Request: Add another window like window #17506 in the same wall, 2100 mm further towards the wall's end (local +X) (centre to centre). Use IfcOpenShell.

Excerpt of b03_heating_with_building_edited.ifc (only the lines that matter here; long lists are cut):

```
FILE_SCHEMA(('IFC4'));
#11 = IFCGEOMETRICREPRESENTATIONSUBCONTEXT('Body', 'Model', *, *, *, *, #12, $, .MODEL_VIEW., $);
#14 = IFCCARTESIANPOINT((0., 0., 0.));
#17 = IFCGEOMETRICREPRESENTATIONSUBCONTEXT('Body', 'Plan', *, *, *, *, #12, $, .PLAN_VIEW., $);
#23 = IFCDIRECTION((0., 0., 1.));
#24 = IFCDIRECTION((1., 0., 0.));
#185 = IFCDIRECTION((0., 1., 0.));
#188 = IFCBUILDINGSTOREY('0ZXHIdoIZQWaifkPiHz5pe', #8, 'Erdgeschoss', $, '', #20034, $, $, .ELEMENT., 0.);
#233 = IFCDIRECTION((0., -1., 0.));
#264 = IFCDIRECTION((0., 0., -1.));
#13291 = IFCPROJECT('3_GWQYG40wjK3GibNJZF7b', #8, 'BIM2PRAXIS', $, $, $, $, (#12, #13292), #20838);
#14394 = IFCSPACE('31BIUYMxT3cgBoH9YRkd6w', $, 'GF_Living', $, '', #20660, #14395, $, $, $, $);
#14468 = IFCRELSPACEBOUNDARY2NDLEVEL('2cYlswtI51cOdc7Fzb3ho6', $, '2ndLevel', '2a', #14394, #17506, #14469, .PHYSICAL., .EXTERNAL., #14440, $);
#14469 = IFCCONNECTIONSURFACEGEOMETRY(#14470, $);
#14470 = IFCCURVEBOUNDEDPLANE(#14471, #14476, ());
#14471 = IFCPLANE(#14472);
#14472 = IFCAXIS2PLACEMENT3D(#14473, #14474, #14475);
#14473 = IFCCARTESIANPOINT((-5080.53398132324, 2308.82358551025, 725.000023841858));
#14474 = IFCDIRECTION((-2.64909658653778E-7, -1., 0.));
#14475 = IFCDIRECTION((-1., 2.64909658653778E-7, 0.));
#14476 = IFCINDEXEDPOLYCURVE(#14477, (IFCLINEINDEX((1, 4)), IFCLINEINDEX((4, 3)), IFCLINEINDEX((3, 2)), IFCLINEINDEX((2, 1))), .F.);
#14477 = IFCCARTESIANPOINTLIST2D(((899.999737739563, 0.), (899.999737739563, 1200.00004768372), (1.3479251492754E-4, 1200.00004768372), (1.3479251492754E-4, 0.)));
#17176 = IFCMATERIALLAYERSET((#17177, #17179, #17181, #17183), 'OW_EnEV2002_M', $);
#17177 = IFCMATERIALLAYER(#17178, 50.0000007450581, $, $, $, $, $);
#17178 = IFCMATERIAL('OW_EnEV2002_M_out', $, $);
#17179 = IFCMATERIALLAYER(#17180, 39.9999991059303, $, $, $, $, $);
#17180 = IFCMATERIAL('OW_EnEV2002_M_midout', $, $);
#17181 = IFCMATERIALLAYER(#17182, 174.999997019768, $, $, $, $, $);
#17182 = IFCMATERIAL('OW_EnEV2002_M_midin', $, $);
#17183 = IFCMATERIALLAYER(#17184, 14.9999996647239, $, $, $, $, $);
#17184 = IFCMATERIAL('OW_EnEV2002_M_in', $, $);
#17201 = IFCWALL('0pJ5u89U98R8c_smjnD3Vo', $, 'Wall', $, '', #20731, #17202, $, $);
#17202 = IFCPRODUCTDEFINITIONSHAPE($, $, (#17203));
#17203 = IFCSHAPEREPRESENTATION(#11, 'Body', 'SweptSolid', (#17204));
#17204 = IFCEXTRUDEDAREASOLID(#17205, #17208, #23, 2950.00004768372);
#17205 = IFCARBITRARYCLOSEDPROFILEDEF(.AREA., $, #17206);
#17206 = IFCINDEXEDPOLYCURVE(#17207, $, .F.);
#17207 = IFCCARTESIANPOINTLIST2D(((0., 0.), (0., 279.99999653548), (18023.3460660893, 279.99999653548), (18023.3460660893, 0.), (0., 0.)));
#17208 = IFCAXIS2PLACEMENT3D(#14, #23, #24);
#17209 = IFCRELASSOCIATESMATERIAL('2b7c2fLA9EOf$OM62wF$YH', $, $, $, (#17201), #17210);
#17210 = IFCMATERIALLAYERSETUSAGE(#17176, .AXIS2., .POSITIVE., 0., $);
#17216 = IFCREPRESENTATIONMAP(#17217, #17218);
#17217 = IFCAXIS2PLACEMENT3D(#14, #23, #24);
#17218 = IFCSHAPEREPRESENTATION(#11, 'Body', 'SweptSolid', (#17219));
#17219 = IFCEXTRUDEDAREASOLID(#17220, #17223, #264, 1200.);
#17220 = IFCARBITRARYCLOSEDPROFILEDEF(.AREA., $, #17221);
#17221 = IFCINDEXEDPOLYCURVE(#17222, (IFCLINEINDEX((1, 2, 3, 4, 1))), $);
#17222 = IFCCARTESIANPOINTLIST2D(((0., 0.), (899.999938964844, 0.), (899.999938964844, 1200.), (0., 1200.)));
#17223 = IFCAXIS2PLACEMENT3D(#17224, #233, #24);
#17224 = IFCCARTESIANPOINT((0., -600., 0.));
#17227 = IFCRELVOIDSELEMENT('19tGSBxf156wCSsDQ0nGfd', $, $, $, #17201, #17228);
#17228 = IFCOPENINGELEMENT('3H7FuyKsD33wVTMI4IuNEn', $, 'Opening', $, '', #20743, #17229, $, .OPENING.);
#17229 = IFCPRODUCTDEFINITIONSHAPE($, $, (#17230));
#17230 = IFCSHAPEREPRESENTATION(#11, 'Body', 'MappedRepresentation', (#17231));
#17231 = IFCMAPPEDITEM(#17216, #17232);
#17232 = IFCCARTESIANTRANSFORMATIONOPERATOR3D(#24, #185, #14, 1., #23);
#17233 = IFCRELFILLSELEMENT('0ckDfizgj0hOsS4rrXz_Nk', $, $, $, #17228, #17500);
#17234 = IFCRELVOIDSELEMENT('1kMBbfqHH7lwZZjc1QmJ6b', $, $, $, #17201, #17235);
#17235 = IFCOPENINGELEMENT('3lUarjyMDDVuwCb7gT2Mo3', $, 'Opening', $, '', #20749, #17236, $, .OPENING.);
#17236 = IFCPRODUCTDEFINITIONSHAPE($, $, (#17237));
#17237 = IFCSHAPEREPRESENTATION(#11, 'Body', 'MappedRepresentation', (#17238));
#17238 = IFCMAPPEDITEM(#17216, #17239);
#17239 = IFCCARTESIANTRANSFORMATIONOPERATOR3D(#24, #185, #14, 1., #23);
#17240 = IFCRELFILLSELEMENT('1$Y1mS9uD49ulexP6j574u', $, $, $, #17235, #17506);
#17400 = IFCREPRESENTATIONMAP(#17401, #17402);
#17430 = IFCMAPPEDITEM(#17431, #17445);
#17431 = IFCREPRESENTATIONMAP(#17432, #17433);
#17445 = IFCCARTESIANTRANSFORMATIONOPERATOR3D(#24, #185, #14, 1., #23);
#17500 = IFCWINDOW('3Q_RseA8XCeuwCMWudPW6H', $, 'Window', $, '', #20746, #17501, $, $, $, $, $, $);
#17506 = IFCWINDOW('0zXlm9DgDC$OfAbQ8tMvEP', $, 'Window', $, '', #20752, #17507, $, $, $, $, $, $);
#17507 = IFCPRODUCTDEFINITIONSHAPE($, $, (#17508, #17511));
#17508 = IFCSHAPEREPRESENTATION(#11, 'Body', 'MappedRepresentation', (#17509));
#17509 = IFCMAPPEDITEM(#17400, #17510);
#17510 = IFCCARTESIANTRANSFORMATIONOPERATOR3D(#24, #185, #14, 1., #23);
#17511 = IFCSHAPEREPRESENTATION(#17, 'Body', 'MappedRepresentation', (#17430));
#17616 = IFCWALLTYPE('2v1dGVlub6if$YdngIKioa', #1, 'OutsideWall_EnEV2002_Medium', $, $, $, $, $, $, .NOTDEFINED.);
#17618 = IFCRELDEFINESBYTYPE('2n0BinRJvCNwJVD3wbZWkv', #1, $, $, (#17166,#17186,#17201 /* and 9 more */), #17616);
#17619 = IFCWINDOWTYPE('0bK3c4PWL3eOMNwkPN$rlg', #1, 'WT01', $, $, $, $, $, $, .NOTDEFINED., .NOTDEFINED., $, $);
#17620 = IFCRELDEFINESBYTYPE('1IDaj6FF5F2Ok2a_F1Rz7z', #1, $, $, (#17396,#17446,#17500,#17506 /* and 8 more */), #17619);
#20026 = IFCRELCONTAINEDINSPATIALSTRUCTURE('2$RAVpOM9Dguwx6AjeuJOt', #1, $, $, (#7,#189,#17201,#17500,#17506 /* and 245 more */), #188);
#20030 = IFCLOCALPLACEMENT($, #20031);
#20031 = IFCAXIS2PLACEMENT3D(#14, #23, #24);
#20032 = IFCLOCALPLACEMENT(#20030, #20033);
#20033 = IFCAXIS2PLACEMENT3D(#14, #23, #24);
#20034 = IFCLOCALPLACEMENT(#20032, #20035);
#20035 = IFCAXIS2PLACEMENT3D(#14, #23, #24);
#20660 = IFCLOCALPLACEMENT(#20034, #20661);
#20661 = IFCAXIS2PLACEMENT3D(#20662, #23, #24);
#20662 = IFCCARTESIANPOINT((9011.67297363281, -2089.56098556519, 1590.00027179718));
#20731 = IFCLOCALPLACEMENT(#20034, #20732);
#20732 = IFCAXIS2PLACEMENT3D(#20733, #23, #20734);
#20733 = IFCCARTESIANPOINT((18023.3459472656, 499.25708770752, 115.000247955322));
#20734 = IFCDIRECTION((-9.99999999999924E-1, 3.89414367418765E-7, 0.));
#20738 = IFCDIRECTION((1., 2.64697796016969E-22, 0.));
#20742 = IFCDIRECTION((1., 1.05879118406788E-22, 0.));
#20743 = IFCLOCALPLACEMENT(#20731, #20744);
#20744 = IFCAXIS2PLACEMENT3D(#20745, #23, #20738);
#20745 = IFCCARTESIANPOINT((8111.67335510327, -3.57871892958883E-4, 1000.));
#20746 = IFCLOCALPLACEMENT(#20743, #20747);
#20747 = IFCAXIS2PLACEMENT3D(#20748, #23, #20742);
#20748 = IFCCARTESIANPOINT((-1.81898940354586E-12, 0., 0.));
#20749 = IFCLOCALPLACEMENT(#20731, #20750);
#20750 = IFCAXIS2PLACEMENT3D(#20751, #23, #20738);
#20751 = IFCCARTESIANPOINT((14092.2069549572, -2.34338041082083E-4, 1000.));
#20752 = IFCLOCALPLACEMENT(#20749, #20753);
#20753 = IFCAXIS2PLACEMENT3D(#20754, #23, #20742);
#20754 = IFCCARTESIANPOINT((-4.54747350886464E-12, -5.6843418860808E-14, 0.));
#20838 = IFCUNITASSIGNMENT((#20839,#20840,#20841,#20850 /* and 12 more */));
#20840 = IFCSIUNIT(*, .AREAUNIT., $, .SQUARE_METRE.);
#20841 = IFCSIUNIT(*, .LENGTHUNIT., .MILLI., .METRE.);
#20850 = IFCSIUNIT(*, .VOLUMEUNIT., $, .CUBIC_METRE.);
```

```python
import numpy as np
import ifcopenshell
import ifcopenshell.api.feature
import ifcopenshell.api.geometry
import ifcopenshell.api.root
import ifcopenshell.geom
import ifcopenshell.util.element
import ifcopenshell.util.placement
import ifcopenshell.util.shape
import ifcopenshell.util.unit

model = ifcopenshell.open("b03_heating_with_building_edited.ifc")
unit_scale = ifcopenshell.util.unit.calculate_unit_scale(model)
settings = ifcopenshell.geom.settings()


def volume(element):
    """Net volume in cubic metres, openings subtracted."""
    shape = ifcopenshell.geom.create_shape(settings, element)
    return ifcopenshell.util.shape.get_volume(shape.geometry)


def reuse_history(source, copy):
    """copy_class also copies each property set's owner history, people and application; keep the originals."""
    for rel in copy.IsDefinedBy:
        if rel.is_a("IfcRelDefinesByProperties") and (history := rel.RelatingPropertyDefinition.OwnerHistory):
            rel.RelatingPropertyDefinition.OwnerHistory = source.OwnerHistory
            ifcopenshell.util.element.remove_deep2(model, history)


window = model.by_guid("0zXlm9DgDC$OfAbQ8tMvEP")
opening = window.FillsVoids[0].RelatingOpeningElement
wall = opening.VoidsElements[0].RelatingBuildingElement
before = volume(wall)
shift = ifcopenshell.util.placement.get_local_placement(wall.ObjectPlacement)[:3, 0] * 2.1 / unit_scale

# copy_class copies the void relationship, type, container and properties, but no geometry.
new_opening = ifcopenshell.api.root.copy_class(model, product=opening)
new_opening.Representation = ifcopenshell.util.element.copy_deep(
    model, opening.Representation, exclude=["IfcGeometricRepresentationContext", "IfcRepresentationMap"]
)
reuse_history(opening, new_opening)
new_window = ifcopenshell.api.root.copy_class(model, product=window)
new_window.Representation = ifcopenshell.util.element.copy_deep(
    model, window.Representation, exclude=["IfcGeometricRepresentationContext", "IfcRepresentationMap"]
)
reuse_history(window, new_window)
ifcopenshell.api.feature.add_filling(model, opening=new_opening, element=new_window)

for old, new in ((opening, new_opening), (window, new_window)):
    matrix = ifcopenshell.util.placement.get_local_placement(old.ObjectPlacement)
    matrix[:3, 3] += shift
    ifcopenshell.api.geometry.edit_object_placement(model, product=new, matrix=matrix, is_si=False)

# The copied space boundaries still share their surfaces with the original.
for rel in new_window.ProvidesBoundaries:
    if rel.ConnectionGeometry:
        rel.ConnectionGeometry = ifcopenshell.util.element.copy_deep(model, rel.ConnectionGeometry)

# Space boundary surfaces are stored in each space's coordinates; move them too.
for rel in new_window.ProvidesBoundaries:
    if not rel.ConnectionGeometry:
        continue
    surface = rel.ConnectionGeometry.SurfaceOnRelatingElement.BasisSurface
    space_matrix = ifcopenshell.util.placement.get_local_placement(rel.RelatingSpace.ObjectPlacement)
    point = np.array(surface.Position.Location.Coordinates) + space_matrix[:3, :3].T @ shift
    surface.Position = model.createIfcAxis2Placement3D(
        model.createIfcCartesianPoint(point.tolist()), surface.Position.Axis, surface.Position.RefDirection
    )

after = volume(wall)

print(f"wall volume {before:.3f} -> {after:.3f} m3")

model.write("b03_heating_with_building_edited_edited.ifc")
```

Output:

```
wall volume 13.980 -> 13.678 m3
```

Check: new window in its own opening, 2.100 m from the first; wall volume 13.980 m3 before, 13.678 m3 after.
